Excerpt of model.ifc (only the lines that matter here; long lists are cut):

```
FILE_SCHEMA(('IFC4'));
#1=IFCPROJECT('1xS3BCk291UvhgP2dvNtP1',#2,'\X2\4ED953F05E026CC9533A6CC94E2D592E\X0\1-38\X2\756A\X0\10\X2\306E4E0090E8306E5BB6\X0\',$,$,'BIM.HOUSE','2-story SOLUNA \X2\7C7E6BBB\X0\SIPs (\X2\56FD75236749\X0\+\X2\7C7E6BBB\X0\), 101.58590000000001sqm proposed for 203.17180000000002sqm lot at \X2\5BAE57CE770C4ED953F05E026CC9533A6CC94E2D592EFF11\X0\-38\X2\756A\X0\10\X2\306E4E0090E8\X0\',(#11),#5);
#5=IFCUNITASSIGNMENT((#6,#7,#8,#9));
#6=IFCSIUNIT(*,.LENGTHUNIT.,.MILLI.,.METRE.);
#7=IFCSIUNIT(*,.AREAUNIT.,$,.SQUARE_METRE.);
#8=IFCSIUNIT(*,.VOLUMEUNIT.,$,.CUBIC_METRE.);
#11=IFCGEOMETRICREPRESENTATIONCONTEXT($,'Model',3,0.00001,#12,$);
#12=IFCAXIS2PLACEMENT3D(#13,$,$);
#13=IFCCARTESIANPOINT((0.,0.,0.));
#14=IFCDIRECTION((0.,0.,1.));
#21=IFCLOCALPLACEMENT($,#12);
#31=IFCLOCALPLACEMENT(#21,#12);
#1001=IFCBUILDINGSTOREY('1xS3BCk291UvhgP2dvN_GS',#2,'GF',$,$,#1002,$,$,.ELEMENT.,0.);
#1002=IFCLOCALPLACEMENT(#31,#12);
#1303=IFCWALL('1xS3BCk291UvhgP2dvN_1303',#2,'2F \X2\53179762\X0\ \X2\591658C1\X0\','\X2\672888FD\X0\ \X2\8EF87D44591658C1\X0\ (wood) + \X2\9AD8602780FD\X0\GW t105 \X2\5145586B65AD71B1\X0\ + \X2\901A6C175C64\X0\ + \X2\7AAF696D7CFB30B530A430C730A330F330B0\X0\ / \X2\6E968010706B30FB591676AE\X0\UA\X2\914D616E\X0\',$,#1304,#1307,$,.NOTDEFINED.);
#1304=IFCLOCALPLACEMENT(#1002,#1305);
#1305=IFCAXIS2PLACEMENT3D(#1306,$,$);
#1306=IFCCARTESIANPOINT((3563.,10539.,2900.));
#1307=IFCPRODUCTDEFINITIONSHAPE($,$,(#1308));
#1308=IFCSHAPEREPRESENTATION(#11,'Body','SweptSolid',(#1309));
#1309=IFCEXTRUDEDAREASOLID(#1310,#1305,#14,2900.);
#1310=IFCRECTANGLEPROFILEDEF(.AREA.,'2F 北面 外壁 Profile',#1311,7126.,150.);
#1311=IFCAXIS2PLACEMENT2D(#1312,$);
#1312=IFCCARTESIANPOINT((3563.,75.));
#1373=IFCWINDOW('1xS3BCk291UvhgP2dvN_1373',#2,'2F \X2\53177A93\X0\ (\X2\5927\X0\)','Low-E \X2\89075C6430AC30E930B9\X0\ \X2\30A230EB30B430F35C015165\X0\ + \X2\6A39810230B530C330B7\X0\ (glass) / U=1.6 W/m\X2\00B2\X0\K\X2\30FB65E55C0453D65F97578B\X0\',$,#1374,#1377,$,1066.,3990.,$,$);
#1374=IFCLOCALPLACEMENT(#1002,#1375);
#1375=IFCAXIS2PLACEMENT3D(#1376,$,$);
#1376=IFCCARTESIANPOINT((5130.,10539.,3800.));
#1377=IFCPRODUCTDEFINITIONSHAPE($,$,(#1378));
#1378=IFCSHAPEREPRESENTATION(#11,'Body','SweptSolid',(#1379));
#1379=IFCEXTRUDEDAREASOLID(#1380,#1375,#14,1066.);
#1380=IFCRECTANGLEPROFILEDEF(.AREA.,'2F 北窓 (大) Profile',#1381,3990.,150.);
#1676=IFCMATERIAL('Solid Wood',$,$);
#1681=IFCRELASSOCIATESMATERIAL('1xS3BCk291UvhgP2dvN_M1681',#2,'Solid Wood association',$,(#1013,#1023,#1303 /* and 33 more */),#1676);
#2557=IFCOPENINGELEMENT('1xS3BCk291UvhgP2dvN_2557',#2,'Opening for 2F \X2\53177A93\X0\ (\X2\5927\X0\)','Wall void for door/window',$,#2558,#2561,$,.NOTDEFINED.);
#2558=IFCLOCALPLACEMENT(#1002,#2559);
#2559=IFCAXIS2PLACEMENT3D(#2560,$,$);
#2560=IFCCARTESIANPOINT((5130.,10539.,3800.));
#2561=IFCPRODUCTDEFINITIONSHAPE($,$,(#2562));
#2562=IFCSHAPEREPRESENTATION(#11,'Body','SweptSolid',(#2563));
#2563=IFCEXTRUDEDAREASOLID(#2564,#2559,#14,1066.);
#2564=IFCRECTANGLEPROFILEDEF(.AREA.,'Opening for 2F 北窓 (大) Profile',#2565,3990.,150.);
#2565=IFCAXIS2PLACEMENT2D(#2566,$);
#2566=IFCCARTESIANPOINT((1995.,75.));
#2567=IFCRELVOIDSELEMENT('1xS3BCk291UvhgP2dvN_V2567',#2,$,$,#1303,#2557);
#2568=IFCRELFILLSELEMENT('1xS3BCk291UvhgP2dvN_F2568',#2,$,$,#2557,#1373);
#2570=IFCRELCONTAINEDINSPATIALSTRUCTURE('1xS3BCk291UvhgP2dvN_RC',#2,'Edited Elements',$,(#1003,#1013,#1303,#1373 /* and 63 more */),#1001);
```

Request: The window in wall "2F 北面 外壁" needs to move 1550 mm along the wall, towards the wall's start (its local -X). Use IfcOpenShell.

```python
import ifcopenshell
import ifcopenshell.api.geometry
import ifcopenshell.util.placement
import ifcopenshell.util.unit

model = ifcopenshell.open("model.ifc")
unit_scale = ifcopenshell.util.unit.calculate_unit_scale(model)

window = model.by_id(1373)
opening = window.FillsVoids[0].RelatingOpeningElement
wall = opening.VoidsElements[0].RelatingBuildingElement

wall_matrix = ifcopenshell.util.placement.get_local_placement(wall.ObjectPlacement)
shift = wall_matrix[:3, 0] * -1.55 / unit_scale
before = ifcopenshell.util.placement.get_local_placement(window.ObjectPlacement)[:3, 3].copy()

# The window is not placed relative to its opening, so move both.
for product in (opening, window):
    matrix = ifcopenshell.util.placement.get_local_placement(product.ObjectPlacement)
    matrix[:3, 3] += shift
    ifcopenshell.api.geometry.edit_object_placement(model, product=product, matrix=matrix, is_si=False)

after = ifcopenshell.util.placement.get_local_placement(window.ObjectPlacement)[:3, 3]
print("window moved by", (after - before).round(3) + 0.0)

model.write("model_edited.ifc")
```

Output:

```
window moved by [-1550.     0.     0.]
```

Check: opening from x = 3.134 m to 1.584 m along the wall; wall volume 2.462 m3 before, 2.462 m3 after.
